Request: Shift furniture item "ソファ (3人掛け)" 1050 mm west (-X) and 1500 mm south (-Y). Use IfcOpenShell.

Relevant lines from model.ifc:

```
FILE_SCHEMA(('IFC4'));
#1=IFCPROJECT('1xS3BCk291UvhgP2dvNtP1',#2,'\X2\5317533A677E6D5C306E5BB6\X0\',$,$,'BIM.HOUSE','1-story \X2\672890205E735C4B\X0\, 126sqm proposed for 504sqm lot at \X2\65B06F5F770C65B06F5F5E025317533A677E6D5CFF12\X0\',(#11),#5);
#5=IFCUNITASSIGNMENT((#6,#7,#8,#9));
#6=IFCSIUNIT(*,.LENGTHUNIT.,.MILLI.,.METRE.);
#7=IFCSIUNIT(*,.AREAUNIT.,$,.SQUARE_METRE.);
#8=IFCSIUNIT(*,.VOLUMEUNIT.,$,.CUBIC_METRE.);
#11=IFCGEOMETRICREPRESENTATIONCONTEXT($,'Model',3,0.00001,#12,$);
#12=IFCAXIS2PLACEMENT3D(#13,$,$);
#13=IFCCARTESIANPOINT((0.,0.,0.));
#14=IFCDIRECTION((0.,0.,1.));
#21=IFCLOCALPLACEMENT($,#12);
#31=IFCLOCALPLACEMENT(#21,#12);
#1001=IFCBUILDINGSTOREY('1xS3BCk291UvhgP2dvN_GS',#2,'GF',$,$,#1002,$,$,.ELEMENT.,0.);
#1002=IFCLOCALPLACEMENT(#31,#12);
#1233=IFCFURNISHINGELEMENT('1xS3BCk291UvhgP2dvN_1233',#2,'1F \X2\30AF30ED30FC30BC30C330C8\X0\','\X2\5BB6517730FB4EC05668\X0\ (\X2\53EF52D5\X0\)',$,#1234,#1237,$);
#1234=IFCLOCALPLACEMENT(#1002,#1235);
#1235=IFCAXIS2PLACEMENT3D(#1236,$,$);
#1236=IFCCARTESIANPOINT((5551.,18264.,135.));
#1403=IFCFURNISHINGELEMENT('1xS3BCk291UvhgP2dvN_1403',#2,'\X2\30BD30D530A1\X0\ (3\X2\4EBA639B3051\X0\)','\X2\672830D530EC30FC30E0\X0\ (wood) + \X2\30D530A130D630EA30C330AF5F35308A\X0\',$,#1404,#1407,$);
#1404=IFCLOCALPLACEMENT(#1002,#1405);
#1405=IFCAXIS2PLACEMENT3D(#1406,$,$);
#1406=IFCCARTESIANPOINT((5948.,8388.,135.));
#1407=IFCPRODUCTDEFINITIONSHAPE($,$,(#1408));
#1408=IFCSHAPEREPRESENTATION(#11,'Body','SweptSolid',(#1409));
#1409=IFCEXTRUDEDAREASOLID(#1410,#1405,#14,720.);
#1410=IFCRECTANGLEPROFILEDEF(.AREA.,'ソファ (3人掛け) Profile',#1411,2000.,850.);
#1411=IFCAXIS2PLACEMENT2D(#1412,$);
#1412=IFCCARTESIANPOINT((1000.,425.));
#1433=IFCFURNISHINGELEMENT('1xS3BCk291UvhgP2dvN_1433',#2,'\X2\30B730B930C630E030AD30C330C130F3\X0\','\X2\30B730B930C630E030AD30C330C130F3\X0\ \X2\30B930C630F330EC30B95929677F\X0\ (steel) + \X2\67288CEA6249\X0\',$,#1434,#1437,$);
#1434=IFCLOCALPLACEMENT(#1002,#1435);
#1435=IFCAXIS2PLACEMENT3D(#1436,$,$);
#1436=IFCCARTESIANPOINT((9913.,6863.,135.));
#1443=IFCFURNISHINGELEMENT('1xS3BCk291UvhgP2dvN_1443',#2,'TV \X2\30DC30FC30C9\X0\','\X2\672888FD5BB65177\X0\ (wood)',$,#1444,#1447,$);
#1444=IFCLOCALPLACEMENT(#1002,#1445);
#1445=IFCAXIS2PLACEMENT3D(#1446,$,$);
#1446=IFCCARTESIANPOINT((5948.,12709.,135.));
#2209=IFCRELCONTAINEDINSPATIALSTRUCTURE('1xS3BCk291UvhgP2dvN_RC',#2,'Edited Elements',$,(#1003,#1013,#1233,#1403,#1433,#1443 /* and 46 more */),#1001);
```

```python
import ifcopenshell
import ifcopenshell.api.geometry
import ifcopenshell.util.placement

model = ifcopenshell.open("model.ifc")

item = model.by_guid("1xS3BCk291UvhgP2dvN_1403")
matrix = ifcopenshell.util.placement.get_local_placement(item.ObjectPlacement)
matrix[0, 3] -= 1050.0
matrix[1, 3] -= 1500.0
ifcopenshell.api.geometry.edit_object_placement(model, product=item, matrix=matrix, is_si=False)

print(ifcopenshell.util.placement.get_local_placement(item.ObjectPlacement).round(3) + 0.0)

model.write("model_edited.ifc")
```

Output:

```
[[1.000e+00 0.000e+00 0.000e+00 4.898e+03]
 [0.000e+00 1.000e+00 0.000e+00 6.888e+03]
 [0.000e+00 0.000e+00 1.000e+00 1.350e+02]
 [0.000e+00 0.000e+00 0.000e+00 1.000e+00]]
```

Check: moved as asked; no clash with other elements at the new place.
